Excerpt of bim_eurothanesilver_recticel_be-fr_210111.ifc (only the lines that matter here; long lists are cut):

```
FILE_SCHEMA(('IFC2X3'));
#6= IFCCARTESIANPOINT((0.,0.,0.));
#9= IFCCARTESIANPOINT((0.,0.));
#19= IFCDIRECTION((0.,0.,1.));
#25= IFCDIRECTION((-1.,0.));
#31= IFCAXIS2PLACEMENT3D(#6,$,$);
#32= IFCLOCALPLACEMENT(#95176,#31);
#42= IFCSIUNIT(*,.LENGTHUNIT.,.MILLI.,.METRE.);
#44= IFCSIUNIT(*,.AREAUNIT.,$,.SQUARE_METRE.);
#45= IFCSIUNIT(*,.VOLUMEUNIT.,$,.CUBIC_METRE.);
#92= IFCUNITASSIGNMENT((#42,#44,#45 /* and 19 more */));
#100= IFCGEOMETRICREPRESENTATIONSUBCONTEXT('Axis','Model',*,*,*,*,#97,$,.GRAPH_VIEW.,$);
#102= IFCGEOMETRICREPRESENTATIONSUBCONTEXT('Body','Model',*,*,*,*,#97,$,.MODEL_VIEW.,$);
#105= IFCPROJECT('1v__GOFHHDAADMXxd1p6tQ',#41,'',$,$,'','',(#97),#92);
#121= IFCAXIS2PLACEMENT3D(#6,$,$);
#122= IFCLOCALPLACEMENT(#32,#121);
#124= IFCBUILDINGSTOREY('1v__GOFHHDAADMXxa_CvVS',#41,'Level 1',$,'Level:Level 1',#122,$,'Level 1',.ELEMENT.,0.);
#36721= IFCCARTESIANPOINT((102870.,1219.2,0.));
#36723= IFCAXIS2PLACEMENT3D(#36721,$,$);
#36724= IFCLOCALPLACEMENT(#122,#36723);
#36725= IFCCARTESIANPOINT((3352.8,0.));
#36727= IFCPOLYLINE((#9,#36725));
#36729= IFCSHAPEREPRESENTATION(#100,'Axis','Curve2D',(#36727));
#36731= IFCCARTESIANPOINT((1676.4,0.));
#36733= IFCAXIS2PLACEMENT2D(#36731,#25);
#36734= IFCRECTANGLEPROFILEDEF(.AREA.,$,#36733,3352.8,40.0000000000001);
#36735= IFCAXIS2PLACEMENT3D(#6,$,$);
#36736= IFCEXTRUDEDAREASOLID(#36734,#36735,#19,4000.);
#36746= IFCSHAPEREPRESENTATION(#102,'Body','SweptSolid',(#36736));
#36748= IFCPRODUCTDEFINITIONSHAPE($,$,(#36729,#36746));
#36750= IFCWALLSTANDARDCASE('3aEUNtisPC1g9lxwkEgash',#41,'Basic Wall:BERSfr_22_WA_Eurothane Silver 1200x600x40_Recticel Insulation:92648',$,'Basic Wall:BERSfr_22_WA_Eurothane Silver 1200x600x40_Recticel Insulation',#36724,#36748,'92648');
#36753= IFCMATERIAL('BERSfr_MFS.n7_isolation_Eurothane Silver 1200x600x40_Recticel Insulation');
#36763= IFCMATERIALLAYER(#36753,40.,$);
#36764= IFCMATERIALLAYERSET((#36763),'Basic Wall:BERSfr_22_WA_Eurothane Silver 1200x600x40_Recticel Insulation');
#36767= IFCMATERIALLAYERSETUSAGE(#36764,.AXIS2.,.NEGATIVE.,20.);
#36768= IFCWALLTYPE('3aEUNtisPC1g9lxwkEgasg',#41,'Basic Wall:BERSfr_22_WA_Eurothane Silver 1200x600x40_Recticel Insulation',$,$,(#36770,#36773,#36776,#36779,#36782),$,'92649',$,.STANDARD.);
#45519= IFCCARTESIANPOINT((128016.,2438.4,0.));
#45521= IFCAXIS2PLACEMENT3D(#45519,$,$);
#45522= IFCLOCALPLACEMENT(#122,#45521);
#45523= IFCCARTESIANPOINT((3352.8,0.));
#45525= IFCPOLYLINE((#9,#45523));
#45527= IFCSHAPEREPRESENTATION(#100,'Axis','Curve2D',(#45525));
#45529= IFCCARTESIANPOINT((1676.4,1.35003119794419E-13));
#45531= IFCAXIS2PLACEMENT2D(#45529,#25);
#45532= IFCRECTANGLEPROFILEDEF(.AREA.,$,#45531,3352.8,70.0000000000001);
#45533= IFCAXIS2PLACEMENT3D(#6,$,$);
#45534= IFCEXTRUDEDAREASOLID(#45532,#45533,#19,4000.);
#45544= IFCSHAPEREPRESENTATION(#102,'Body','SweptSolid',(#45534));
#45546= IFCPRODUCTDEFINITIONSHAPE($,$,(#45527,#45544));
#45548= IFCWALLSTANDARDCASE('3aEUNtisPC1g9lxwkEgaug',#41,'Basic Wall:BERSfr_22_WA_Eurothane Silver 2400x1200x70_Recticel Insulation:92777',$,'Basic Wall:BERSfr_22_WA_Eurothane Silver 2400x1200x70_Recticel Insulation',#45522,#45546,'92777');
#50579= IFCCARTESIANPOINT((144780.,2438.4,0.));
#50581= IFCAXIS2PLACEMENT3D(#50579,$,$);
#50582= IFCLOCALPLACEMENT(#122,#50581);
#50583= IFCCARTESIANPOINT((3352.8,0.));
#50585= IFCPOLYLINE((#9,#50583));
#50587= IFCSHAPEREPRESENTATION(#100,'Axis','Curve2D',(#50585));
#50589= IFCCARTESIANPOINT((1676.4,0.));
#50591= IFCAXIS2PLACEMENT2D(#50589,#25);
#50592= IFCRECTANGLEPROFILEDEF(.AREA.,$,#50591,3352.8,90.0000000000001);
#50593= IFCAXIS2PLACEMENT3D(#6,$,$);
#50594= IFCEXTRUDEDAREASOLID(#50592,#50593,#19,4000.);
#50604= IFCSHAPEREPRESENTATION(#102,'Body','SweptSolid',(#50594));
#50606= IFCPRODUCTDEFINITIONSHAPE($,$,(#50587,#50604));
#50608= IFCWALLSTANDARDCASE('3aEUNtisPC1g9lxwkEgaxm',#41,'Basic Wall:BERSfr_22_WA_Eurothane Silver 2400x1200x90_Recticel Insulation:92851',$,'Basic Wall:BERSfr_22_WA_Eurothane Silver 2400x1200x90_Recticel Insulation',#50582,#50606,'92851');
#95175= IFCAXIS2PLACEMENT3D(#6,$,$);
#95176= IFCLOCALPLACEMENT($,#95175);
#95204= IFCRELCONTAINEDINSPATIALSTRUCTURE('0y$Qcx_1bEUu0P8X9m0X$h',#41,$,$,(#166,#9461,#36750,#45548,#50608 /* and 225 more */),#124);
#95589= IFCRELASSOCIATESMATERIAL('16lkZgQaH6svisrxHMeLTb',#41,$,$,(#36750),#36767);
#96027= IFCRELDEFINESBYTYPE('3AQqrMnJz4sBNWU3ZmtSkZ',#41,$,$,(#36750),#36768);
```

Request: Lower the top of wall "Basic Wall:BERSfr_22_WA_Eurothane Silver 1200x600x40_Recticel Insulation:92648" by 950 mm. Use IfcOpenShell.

```python
import ifcopenshell
import ifcopenshell.geom
import ifcopenshell.util.representation
import ifcopenshell.util.shape

model = ifcopenshell.open("bim_eurothanesilver_recticel_be-fr_210111.ifc")
settings = ifcopenshell.geom.settings()


def volume(element):
    """Net volume in cubic metres, openings subtracted."""
    shape = ifcopenshell.geom.create_shape(settings, element)
    return ifcopenshell.util.shape.get_volume(shape.geometry)


wall = model.by_guid("3aEUNtisPC1g9lxwkEgash")
before = volume(wall)

body = ifcopenshell.util.representation.get_representation(wall, "Model", "Body")
solid = body.Items[0]
old_height = solid.Depth
solid.Depth -= 950.0
after = volume(wall)

print(f"height {old_height:g} -> {solid.Depth:g}, volume {before:.3f} -> {after:.3f} m3")

model.write("bim_eurothanesilver_recticel_be-fr_210111-out.ifc")
```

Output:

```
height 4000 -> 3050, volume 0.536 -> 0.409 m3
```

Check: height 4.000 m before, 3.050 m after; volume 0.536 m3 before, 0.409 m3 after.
